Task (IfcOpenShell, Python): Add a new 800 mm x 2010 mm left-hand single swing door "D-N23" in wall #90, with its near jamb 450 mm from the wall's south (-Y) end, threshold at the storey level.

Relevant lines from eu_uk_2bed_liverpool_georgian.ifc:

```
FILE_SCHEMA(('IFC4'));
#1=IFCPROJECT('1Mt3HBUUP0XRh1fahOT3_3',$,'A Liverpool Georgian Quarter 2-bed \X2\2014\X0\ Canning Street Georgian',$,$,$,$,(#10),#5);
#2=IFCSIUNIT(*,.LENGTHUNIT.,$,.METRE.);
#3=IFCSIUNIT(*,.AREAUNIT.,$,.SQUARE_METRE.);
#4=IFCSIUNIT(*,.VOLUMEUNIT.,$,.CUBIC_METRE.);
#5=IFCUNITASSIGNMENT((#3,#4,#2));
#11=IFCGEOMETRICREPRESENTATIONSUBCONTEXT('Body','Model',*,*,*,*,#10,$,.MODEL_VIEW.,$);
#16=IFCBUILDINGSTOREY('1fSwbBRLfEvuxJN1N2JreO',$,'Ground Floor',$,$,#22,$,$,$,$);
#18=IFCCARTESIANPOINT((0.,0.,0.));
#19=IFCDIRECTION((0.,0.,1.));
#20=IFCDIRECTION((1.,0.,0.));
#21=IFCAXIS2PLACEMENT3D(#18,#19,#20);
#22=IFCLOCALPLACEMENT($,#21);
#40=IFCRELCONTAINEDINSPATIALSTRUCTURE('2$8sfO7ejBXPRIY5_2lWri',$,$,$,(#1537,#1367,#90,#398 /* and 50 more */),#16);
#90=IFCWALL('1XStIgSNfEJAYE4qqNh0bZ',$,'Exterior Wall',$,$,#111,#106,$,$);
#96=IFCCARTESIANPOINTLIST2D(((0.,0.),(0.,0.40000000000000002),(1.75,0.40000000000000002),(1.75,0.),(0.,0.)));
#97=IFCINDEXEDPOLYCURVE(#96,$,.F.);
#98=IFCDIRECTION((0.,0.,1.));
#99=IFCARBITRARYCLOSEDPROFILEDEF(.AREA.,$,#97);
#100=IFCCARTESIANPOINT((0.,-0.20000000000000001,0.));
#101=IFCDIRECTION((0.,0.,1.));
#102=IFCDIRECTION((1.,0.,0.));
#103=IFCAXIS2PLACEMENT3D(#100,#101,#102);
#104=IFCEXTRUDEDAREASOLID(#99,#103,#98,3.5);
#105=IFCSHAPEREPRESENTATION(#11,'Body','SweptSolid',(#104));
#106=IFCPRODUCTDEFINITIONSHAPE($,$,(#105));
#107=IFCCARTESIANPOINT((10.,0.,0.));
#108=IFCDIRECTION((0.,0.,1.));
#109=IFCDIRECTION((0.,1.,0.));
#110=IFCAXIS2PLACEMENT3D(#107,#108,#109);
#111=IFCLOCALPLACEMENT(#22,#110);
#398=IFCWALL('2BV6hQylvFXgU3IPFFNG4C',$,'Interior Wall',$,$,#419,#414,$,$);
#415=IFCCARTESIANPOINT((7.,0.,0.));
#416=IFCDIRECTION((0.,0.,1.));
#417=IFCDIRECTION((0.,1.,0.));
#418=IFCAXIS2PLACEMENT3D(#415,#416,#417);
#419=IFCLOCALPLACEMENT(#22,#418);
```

```python
import numpy as np
import ifcopenshell
import ifcopenshell.api.feature
import ifcopenshell.api.geometry
import ifcopenshell.api.root
import ifcopenshell.api.spatial
import ifcopenshell.geom
import ifcopenshell.util.element
import ifcopenshell.util.placement
import ifcopenshell.util.representation
import ifcopenshell.util.shape
import ifcopenshell.util.unit

model = ifcopenshell.open("eu_uk_2bed_liverpool_georgian.ifc")
unit_scale = ifcopenshell.util.unit.calculate_unit_scale(model)
settings = ifcopenshell.geom.settings()


def volume(element):
    """Net volume in cubic metres, openings subtracted."""
    shape = ifcopenshell.geom.create_shape(settings, element)
    return ifcopenshell.util.shape.get_volume(shape.geometry)


wall = model.by_guid("1XStIgSNfEJAYE4qqNh0bZ")
storey = ifcopenshell.util.element.get_container(wall, ifc_class="IfcBuildingStorey")
context = ifcopenshell.util.representation.get_context(model, "Model", "Body", "MODEL_VIEW")
before = volume(wall)

width, height, from_end, sill = 0.8, 2.01, 0.45, 0.0  # metres

# The wall runs along its own X axis, and the end named is its -X end.
wall_shape = ifcopenshell.geom.create_shape(settings, wall)
x, y, z = ifcopenshell.util.shape.get_vertices(wall_shape.geometry).T
start = x.min() + from_end
face, thickness = float(y.min()), float(y.max() - y.min())
wall_matrix = ifcopenshell.util.placement.get_local_placement(wall.ObjectPlacement)
level = ifcopenshell.util.placement.get_local_placement(storey.ObjectPlacement)[2, 3]


def in_wall(x, y):
    """Placement at x, y metres in the wall's axes, at sill height."""
    matrix = wall_matrix.copy()
    matrix[:, 3] = wall_matrix @ np.array([x / unit_scale, y / unit_scale, 0.0, 1.0])
    matrix[2, 3] = level + sill / unit_scale
    return matrix


# Opening: a box that overshoots both wall faces by 50 mm.
opening = ifcopenshell.api.root.create_entity(model, ifc_class="IfcOpeningElement", predefined_type="OPENING")
box = ifcopenshell.api.geometry.add_wall_representation(
    model, context=context, length=width, height=height, thickness=thickness + 0.1
)
ifcopenshell.api.geometry.assign_representation(model, product=opening, representation=box)
ifcopenshell.api.geometry.edit_object_placement(model, product=opening, matrix=in_wall(start, face - 0.05), is_si=False)
ifcopenshell.api.feature.add_feature(model, feature=opening, element=wall)

door = ifcopenshell.api.root.create_entity(model, ifc_class="IfcDoor", name="D-N23", predefined_type="DOOR")
door.OverallWidth, door.OverallHeight = width / unit_scale, height / unit_scale
door.OperationType = "SINGLE_SWING_LEFT"
body = ifcopenshell.api.geometry.add_door_representation(
    model,
    context=context,
    overall_width=door.OverallWidth,
    overall_height=door.OverallHeight,
    operation_type="SINGLE_SWING_LEFT",
    lining_properties={"LiningDepth": thickness / unit_scale, "ThresholdDepth": thickness / unit_scale},
)
ifcopenshell.api.geometry.assign_representation(model, product=door, representation=body)
ifcopenshell.api.spatial.assign_container(model, products=[door], relating_structure=storey)
ifcopenshell.api.feature.add_filling(model, opening=opening, element=door)

# The lining spans the wall, so the door starts at the wall face.
ifcopenshell.api.geometry.edit_object_placement(model, product=door, matrix=in_wall(start, face), is_si=False)

after = volume(wall)

print(f"wall volume {before:.3f} -> {after:.3f} m3")

model.write("eu_uk_2bed_liverpool_georgian_rev.ifc")
```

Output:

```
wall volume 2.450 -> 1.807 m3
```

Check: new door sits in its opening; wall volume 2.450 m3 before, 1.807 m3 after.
